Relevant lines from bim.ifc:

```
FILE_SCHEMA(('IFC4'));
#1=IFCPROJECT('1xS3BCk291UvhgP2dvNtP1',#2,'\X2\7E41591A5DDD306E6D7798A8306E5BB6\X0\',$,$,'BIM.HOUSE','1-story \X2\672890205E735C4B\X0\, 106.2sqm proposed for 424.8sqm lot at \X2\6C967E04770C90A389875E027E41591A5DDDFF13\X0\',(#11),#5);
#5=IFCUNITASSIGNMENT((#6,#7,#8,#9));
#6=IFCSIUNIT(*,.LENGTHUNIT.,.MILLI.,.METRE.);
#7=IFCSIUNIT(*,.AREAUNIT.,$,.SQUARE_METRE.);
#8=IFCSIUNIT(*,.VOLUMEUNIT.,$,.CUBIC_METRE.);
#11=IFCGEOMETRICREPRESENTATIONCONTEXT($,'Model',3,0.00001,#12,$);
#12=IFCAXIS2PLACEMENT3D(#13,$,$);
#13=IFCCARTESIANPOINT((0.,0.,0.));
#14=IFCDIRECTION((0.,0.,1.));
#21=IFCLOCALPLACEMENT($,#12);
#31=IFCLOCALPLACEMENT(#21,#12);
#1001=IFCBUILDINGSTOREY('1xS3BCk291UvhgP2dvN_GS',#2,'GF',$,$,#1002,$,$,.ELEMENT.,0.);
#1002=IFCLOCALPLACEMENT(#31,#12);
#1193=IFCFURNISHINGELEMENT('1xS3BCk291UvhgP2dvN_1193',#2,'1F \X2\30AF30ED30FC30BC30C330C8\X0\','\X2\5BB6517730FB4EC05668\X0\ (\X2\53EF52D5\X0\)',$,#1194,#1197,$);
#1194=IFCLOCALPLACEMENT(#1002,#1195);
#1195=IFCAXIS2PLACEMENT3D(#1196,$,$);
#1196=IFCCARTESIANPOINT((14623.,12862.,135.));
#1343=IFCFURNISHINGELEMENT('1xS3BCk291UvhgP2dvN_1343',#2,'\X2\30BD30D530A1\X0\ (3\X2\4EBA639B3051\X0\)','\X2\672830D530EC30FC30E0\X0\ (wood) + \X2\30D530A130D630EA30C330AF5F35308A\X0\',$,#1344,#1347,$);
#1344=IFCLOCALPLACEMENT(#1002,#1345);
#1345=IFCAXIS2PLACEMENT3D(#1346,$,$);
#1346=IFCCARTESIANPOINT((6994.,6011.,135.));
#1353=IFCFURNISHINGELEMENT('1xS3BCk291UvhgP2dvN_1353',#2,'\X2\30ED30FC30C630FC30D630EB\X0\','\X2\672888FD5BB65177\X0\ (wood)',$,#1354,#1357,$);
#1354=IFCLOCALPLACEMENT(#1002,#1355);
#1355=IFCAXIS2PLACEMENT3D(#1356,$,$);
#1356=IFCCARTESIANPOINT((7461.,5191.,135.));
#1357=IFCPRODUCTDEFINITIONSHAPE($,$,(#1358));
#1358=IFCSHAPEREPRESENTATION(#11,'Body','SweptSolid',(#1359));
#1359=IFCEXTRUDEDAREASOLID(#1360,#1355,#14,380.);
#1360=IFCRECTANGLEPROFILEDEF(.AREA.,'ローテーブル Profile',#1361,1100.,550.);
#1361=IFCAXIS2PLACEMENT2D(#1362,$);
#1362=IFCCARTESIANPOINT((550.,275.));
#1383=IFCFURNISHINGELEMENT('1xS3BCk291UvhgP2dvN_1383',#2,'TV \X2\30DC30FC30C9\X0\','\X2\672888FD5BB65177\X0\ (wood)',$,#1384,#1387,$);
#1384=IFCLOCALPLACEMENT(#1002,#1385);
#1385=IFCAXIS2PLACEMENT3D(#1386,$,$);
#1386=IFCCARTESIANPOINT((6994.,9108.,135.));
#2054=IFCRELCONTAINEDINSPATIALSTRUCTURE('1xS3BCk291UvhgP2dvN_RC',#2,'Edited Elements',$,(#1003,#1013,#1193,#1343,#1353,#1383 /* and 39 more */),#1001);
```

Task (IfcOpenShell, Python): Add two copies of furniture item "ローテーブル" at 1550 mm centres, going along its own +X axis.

```python
import ifcopenshell
import ifcopenshell.api.geometry
import ifcopenshell.api.root
import ifcopenshell.util.element
import ifcopenshell.util.placement

model = ifcopenshell.open("bim.ifc")


def reuse_history(source, copy):
    """copy_class also copies each property set's owner history, people and application; keep the originals."""
    for rel in copy.IsDefinedBy:
        if rel.is_a("IfcRelDefinesByProperties") and (history := rel.RelatingPropertyDefinition.OwnerHistory):
            rel.RelatingPropertyDefinition.OwnerHistory = source.OwnerHistory
            ifcopenshell.util.element.remove_deep2(model, history)


source = model.by_guid("1xS3BCk291UvhgP2dvN_1353")
base = ifcopenshell.util.placement.get_local_placement(source.ObjectPlacement)
step = base[:3, 0] * 1550.0

for i in range(1, 3):
    copy = ifcopenshell.api.root.copy_class(model, product=source)
    copy.Representation = ifcopenshell.util.element.copy_deep(
        model, source.Representation, exclude=["IfcGeometricRepresentationContext", "IfcRepresentationMap"]
    )
    reuse_history(source, copy)
    matrix = base.copy()
    matrix[:3, 3] += i * step
    print("added at", matrix[:3, 3].round(3) + 0.0)
    ifcopenshell.api.geometry.edit_object_placement(model, product=copy, matrix=matrix, is_si=False)

model.write("bim_v2.ifc")
```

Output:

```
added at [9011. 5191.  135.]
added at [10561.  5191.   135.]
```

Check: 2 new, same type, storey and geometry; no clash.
